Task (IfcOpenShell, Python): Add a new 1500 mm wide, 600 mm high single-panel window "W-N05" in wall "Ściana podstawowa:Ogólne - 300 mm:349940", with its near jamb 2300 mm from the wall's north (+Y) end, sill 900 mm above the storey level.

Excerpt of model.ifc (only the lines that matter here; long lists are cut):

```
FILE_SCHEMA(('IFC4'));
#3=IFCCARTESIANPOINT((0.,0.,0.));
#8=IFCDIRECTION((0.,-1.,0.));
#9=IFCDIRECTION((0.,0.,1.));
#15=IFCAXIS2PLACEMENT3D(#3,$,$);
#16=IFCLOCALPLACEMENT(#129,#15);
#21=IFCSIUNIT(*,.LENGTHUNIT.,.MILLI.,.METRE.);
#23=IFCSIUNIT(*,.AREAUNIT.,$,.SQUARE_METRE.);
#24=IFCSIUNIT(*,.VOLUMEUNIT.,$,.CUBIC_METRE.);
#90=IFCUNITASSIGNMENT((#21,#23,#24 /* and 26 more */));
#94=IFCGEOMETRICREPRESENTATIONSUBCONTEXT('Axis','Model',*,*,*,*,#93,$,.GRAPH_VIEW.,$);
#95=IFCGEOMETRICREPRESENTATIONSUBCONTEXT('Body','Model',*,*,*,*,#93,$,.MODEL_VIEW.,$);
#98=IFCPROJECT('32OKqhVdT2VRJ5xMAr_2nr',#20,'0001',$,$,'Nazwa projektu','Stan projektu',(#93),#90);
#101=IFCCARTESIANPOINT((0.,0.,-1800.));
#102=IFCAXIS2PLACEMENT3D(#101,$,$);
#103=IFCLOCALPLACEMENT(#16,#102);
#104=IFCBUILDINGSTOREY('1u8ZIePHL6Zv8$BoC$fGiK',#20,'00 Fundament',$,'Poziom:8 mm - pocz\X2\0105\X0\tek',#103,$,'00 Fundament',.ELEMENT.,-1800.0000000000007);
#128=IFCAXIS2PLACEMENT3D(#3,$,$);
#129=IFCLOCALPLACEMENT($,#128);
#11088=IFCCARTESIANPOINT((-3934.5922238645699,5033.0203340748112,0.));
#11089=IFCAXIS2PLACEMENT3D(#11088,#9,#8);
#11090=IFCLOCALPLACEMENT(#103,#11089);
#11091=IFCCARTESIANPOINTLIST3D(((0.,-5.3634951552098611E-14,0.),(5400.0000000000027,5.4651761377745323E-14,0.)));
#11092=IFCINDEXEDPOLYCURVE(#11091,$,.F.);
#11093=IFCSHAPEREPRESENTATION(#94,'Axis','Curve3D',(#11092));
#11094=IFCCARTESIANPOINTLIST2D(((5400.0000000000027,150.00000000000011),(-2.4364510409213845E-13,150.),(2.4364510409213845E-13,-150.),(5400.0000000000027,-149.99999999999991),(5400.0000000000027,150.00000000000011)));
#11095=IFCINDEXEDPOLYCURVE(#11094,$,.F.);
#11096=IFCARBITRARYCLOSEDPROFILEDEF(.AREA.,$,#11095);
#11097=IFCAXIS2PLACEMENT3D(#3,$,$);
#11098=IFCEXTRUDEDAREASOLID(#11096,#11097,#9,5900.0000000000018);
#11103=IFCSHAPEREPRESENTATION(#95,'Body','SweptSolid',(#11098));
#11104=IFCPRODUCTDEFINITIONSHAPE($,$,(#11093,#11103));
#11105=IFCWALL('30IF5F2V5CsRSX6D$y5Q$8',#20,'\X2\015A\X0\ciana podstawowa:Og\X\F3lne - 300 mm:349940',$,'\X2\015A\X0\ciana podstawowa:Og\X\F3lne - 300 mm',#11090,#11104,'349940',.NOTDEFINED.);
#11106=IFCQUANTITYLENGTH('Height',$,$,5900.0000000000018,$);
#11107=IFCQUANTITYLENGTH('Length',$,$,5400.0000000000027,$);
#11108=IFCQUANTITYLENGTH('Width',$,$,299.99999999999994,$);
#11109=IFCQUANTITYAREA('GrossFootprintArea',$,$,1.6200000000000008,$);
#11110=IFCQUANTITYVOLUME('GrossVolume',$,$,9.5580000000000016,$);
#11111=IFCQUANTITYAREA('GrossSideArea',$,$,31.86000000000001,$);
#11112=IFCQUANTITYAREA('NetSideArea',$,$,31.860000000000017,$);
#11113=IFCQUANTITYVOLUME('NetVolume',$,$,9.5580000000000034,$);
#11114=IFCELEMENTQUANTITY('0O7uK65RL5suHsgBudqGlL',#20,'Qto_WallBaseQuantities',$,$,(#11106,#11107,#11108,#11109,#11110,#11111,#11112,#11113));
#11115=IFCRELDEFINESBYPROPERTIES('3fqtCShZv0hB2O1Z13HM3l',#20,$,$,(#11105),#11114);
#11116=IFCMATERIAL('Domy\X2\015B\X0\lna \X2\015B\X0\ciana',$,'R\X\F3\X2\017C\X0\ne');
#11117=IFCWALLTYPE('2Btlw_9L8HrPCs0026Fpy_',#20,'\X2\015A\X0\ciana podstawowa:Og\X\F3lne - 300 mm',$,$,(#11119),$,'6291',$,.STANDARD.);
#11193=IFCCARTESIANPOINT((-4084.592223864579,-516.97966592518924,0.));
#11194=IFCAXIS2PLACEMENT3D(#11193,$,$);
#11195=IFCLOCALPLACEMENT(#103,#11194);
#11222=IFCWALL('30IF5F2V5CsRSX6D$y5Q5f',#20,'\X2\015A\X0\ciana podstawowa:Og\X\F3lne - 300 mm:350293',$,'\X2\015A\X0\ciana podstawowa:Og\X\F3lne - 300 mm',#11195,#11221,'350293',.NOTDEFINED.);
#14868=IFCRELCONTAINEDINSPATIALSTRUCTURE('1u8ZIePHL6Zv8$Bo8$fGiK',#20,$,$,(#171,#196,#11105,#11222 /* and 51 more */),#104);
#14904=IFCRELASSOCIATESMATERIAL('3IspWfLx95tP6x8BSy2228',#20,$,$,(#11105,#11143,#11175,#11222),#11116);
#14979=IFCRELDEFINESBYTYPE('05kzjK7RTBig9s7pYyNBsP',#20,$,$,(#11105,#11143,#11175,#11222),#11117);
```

```python
import numpy as np
import ifcopenshell
import ifcopenshell.api.feature
import ifcopenshell.api.geometry
import ifcopenshell.api.pset
import ifcopenshell.api.root
import ifcopenshell.api.spatial
import ifcopenshell.geom
import ifcopenshell.util.element
import ifcopenshell.util.placement
import ifcopenshell.util.representation
import ifcopenshell.util.shape
import ifcopenshell.util.unit

model = ifcopenshell.open("model.ifc")
unit_scale = ifcopenshell.util.unit.calculate_unit_scale(model)
area_scale = ifcopenshell.util.unit.calculate_unit_scale(model, "AREAUNIT")
volume_scale = ifcopenshell.util.unit.calculate_unit_scale(model, "VOLUMEUNIT")
settings = ifcopenshell.geom.settings()


def volume(element):
    """Net volume in cubic metres, openings subtracted."""
    shape = ifcopenshell.geom.create_shape(settings, element)
    return ifcopenshell.util.shape.get_volume(shape.geometry)


wall = model.by_guid("30IF5F2V5CsRSX6D$y5Q$8")
storey = ifcopenshell.util.element.get_container(wall, ifc_class="IfcBuildingStorey")
context = ifcopenshell.util.representation.get_context(model, "Model", "Body", "MODEL_VIEW")
before = volume(wall)

width, height, from_end, sill = 1.5, 0.6, 2.3, 0.9  # metres

# The wall runs along its own X axis, and the end named is its -X end.
wall_shape = ifcopenshell.geom.create_shape(settings, wall)
x, y, z = ifcopenshell.util.shape.get_vertices(wall_shape.geometry).T
start = x.min() + from_end
face, thickness = float(y.min()), float(y.max() - y.min())
wall_matrix = ifcopenshell.util.placement.get_local_placement(wall.ObjectPlacement)
level = ifcopenshell.util.placement.get_local_placement(storey.ObjectPlacement)[2, 3]


def in_wall(x, y):
    """Placement at x, y metres in the wall's axes, at sill height."""
    matrix = wall_matrix.copy()
    matrix[:, 3] = wall_matrix @ np.array([x / unit_scale, y / unit_scale, 0.0, 1.0])
    matrix[2, 3] = level + sill / unit_scale
    return matrix


# Opening: a box that overshoots both wall faces by 50 mm.
opening = ifcopenshell.api.root.create_entity(model, ifc_class="IfcOpeningElement", predefined_type="OPENING")
box = ifcopenshell.api.geometry.add_wall_representation(
    model, context=context, length=width, height=height, thickness=thickness + 0.1
)
ifcopenshell.api.geometry.assign_representation(model, product=opening, representation=box)
ifcopenshell.api.geometry.edit_object_placement(model, product=opening, matrix=in_wall(start, face - 0.05), is_si=False)
ifcopenshell.api.feature.add_feature(model, feature=opening, element=wall)

window = ifcopenshell.api.root.create_entity(model, ifc_class="IfcWindow", name="W-N05", predefined_type="WINDOW")
window.OverallWidth, window.OverallHeight = width / unit_scale, height / unit_scale
window.PartitioningType = "SINGLE_PANEL"
body = ifcopenshell.api.geometry.add_window_representation(
    model,
    context=context,
    overall_width=window.OverallWidth,
    overall_height=window.OverallHeight,
    partition_type="SINGLE_PANEL",
)
ifcopenshell.api.geometry.assign_representation(model, product=window, representation=body)
ifcopenshell.api.spatial.assign_container(model, products=[window], relating_structure=storey)
ifcopenshell.api.feature.add_filling(model, opening=opening, element=window)

# Centre the window in the wall's thickness.
ifcopenshell.api.geometry.edit_object_placement(model, product=window, matrix=in_wall(start, face), is_si=False)
window_shape = ifcopenshell.geom.create_shape(settings, window)
depth = ifcopenshell.util.shape.get_vertices(window_shape.geometry)[:, 1]
offset = face + thickness / 2 - (depth.min() + depth.max()) / 2
ifcopenshell.api.geometry.edit_object_placement(model, product=window, matrix=in_wall(start, offset), is_si=False)

after = volume(wall)

# Update the wall's stored quantities.
qto = model.by_id(ifcopenshell.util.element.get_pset(wall, "Qto_WallBaseQuantities", should_inherit=False)["id"])
ifcopenshell.api.pset.edit_qto(model, qto=qto, properties={
    "NetSideArea": after / thickness / area_scale,
    "NetVolume": after / volume_scale,
})

print(f"wall volume {before:.3f} -> {after:.3f} m3")

model.write("model_updated.ifc")
```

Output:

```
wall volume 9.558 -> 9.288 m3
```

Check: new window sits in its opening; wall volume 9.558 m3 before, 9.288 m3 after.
